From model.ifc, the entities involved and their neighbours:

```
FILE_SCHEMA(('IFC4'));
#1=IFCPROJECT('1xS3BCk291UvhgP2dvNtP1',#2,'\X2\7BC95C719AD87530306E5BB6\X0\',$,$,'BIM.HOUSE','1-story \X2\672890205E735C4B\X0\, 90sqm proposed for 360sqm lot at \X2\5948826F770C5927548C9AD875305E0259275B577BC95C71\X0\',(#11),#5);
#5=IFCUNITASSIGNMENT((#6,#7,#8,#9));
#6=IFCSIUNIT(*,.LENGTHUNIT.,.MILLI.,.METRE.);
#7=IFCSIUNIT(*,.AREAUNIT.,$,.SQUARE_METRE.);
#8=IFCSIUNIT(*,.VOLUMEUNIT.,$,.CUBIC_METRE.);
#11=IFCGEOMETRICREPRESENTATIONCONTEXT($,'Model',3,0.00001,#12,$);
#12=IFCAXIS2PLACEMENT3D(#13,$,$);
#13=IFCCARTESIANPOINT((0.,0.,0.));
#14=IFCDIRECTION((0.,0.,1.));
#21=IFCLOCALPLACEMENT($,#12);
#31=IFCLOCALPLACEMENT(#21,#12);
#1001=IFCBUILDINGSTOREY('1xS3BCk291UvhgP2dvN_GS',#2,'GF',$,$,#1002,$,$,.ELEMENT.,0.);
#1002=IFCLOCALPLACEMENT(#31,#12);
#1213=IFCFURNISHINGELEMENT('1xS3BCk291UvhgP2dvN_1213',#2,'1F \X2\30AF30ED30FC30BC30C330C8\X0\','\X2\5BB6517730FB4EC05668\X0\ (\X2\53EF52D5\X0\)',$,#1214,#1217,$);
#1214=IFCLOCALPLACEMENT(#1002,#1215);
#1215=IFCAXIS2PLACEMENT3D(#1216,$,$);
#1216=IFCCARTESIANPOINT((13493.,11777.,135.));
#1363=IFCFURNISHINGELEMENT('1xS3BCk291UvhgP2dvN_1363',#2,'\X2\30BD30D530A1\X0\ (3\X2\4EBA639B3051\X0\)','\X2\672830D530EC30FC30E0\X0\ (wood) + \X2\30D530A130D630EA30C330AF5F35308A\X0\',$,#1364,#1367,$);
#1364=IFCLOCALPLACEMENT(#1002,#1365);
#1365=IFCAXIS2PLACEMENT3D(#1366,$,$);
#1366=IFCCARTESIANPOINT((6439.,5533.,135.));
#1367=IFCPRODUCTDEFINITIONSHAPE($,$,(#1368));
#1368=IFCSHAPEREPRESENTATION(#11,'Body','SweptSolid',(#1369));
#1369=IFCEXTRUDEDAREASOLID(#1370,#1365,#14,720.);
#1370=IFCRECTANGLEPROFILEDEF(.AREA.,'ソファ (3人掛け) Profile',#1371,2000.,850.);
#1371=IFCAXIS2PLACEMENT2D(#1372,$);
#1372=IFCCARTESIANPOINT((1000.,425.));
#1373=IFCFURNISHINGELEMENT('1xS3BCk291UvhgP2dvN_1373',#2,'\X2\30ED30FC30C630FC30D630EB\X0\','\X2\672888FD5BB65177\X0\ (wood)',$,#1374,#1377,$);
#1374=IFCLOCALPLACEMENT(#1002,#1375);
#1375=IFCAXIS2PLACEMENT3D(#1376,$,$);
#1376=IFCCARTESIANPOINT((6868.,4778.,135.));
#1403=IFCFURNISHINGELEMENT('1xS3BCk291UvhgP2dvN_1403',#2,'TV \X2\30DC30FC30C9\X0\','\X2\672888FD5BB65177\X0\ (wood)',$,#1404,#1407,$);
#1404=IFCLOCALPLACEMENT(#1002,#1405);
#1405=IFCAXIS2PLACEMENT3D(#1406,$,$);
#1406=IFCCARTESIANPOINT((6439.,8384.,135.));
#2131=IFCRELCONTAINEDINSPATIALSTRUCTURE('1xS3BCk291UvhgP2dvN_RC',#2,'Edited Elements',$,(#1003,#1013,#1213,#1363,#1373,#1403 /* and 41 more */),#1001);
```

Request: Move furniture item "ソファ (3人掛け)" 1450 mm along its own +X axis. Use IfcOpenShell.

```python
import ifcopenshell
import ifcopenshell.api.geometry
import ifcopenshell.util.placement
import ifcopenshell.util.unit

model = ifcopenshell.open("model.ifc")
unit_scale = ifcopenshell.util.unit.calculate_unit_scale(model)

item = model.by_guid("1xS3BCk291UvhgP2dvN_1363")
matrix = ifcopenshell.util.placement.get_local_placement(item.ObjectPlacement)
matrix[:3, 3] += matrix[:3, 0] * 1.45 / unit_scale
ifcopenshell.api.geometry.edit_object_placement(model, product=item, matrix=matrix, is_si=False)

print(ifcopenshell.util.placement.get_local_placement(item.ObjectPlacement).round(3) + 0.0)

model.write("model-out.ifc")
```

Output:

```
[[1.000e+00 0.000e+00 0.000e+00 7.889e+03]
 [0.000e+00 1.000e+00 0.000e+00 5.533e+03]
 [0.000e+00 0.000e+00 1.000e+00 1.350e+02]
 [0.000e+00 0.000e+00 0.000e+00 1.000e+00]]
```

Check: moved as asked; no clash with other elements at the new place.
